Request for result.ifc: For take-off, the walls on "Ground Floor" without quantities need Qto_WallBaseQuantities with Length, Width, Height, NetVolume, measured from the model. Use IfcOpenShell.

First a look at what the model holds.

```python
import ifcopenshell
import ifcopenshell.util.element
import ifcopenshell.util.unit

model = ifcopenshell.open("result.ifc")
print(model.schema)
for unit_type in ("LENGTHUNIT", "AREAUNIT", "VOLUMEUNIT"):
    print(unit_type, ifcopenshell.util.unit.calculate_unit_scale(model, unit_type))
storey = next(s for s in model.by_type("IfcBuildingStorey") if s.Name == "Ground Floor")
walls = [e for e in ifcopenshell.util.element.get_decomposition(storey) if e.is_a("IfcWall")]
for e in sorted(walls, key=lambda e: e.id()):
    print(e.id(), e.is_a(), e.Name, list(ifcopenshell.util.element.get_psets(e, qtos_only=True)), sep=" | ")
```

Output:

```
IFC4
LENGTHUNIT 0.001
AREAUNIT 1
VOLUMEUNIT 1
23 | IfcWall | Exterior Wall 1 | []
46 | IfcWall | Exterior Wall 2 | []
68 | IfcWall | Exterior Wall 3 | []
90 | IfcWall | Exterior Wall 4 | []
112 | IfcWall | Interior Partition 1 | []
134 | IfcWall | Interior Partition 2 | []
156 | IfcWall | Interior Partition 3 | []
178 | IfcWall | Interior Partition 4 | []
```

```python
import ifcopenshell
import ifcopenshell.api.pset
import ifcopenshell.geom
import ifcopenshell.util.element
import ifcopenshell.util.shape
import ifcopenshell.util.unit

model = ifcopenshell.open("result.ifc")
unit_scale = ifcopenshell.util.unit.calculate_unit_scale(model)
volume_scale = ifcopenshell.util.unit.calculate_unit_scale(model, "VOLUMEUNIT")
settings = ifcopenshell.geom.settings()

storey = next(s for s in model.by_type("IfcBuildingStorey") if s.Name == "Ground Floor")
walls = [e for e in ifcopenshell.util.element.get_decomposition(storey) if e.is_a("IfcWall")]

for e in sorted(walls, key=lambda e: e.id()):
    if ifcopenshell.util.element.get_psets(e, qtos_only=True, should_inherit=False):
        continue
    # Geometry comes back in metres, in the element's own axes.
    shape = ifcopenshell.geom.create_shape(settings, e)
    values = {
        "Length": ifcopenshell.util.shape.get_x(shape.geometry) / unit_scale,
        "Width": ifcopenshell.util.shape.get_y(shape.geometry) / unit_scale,
        "Height": ifcopenshell.util.shape.get_z(shape.geometry) / unit_scale,
        "NetVolume": ifcopenshell.util.shape.get_volume(shape.geometry) / volume_scale,
    }
    qto = ifcopenshell.api.pset.add_qto(model, product=e, name="Qto_WallBaseQuantities")
    ifcopenshell.api.pset.edit_qto(model, qto=qto, properties=values)
    print(e.id(), {k: round(v, 3) for k, v in values.items()})

model.write("result_updated.ifc")
```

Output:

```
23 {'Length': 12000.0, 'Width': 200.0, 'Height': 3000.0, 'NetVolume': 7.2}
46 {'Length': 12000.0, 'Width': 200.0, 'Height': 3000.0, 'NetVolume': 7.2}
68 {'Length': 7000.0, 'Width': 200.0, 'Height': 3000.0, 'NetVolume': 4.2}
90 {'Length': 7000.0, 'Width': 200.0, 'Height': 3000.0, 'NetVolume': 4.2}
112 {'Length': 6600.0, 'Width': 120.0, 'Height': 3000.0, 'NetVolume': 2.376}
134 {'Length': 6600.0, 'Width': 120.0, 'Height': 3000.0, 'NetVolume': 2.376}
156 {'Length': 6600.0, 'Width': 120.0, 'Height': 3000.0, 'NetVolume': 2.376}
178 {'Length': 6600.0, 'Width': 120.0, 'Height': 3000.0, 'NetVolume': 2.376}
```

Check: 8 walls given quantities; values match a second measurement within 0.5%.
